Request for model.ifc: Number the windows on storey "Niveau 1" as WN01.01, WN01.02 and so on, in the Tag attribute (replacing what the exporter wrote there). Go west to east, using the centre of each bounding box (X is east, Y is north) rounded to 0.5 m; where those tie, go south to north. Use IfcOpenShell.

First a look at what the model holds.

```python
import ifcopenshell
import ifcopenshell.util.element
import ifcopenshell.util.placement

model = ifcopenshell.open("model.ifc")
print(model.schema)
storey = next(s for s in model.by_type("IfcBuildingStorey") if s.Name == "Niveau 1")
windows = [e for e in ifcopenshell.util.element.get_decomposition(storey) if e.is_a("IfcWindow")]
for e in sorted(windows, key=lambda e: e.id()):
    origin = ifcopenshell.util.placement.get_local_placement(e.ObjectPlacement)[:3, 3]
    print(e.id(), e.Tag, e.Name, origin.round(2) + 0.0, sep=" | ")
```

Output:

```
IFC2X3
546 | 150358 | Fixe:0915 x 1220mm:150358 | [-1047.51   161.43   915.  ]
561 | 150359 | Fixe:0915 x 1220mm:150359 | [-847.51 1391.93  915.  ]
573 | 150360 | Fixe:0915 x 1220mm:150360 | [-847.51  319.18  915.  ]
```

```python
import ifcopenshell
import ifcopenshell.geom
import ifcopenshell.util.element
import ifcopenshell.util.shape

model = ifcopenshell.open("model.ifc")
settings = ifcopenshell.geom.settings()
settings.set("use-world-coords", True)


def centre(element):
    shape = ifcopenshell.geom.create_shape(settings, element)
    return ifcopenshell.util.shape.get_bbox_centroid(shape.geometry)


storey = next(s for s in model.by_type("IfcBuildingStorey") if s.Name == "Niveau 1")
windows = [e for e in ifcopenshell.util.element.get_decomposition(storey) if e.is_a("IfcWindow")]

# Insertion points can sit at a corner or the storey origin, so sort by the geometry (in metres).
centres = {e: centre(e) for e in windows}
windows.sort(key=lambda e: (round(centres[e][0] / 0.5), centres[e][1]))

for i, e in enumerate(windows, start=1):
    number = f"WN01.{i:02d}"
    e.Tag = number
    print(e.id(), number)

model.write("model_rev.ifc")
```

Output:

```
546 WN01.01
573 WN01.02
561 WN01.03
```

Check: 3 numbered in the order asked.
